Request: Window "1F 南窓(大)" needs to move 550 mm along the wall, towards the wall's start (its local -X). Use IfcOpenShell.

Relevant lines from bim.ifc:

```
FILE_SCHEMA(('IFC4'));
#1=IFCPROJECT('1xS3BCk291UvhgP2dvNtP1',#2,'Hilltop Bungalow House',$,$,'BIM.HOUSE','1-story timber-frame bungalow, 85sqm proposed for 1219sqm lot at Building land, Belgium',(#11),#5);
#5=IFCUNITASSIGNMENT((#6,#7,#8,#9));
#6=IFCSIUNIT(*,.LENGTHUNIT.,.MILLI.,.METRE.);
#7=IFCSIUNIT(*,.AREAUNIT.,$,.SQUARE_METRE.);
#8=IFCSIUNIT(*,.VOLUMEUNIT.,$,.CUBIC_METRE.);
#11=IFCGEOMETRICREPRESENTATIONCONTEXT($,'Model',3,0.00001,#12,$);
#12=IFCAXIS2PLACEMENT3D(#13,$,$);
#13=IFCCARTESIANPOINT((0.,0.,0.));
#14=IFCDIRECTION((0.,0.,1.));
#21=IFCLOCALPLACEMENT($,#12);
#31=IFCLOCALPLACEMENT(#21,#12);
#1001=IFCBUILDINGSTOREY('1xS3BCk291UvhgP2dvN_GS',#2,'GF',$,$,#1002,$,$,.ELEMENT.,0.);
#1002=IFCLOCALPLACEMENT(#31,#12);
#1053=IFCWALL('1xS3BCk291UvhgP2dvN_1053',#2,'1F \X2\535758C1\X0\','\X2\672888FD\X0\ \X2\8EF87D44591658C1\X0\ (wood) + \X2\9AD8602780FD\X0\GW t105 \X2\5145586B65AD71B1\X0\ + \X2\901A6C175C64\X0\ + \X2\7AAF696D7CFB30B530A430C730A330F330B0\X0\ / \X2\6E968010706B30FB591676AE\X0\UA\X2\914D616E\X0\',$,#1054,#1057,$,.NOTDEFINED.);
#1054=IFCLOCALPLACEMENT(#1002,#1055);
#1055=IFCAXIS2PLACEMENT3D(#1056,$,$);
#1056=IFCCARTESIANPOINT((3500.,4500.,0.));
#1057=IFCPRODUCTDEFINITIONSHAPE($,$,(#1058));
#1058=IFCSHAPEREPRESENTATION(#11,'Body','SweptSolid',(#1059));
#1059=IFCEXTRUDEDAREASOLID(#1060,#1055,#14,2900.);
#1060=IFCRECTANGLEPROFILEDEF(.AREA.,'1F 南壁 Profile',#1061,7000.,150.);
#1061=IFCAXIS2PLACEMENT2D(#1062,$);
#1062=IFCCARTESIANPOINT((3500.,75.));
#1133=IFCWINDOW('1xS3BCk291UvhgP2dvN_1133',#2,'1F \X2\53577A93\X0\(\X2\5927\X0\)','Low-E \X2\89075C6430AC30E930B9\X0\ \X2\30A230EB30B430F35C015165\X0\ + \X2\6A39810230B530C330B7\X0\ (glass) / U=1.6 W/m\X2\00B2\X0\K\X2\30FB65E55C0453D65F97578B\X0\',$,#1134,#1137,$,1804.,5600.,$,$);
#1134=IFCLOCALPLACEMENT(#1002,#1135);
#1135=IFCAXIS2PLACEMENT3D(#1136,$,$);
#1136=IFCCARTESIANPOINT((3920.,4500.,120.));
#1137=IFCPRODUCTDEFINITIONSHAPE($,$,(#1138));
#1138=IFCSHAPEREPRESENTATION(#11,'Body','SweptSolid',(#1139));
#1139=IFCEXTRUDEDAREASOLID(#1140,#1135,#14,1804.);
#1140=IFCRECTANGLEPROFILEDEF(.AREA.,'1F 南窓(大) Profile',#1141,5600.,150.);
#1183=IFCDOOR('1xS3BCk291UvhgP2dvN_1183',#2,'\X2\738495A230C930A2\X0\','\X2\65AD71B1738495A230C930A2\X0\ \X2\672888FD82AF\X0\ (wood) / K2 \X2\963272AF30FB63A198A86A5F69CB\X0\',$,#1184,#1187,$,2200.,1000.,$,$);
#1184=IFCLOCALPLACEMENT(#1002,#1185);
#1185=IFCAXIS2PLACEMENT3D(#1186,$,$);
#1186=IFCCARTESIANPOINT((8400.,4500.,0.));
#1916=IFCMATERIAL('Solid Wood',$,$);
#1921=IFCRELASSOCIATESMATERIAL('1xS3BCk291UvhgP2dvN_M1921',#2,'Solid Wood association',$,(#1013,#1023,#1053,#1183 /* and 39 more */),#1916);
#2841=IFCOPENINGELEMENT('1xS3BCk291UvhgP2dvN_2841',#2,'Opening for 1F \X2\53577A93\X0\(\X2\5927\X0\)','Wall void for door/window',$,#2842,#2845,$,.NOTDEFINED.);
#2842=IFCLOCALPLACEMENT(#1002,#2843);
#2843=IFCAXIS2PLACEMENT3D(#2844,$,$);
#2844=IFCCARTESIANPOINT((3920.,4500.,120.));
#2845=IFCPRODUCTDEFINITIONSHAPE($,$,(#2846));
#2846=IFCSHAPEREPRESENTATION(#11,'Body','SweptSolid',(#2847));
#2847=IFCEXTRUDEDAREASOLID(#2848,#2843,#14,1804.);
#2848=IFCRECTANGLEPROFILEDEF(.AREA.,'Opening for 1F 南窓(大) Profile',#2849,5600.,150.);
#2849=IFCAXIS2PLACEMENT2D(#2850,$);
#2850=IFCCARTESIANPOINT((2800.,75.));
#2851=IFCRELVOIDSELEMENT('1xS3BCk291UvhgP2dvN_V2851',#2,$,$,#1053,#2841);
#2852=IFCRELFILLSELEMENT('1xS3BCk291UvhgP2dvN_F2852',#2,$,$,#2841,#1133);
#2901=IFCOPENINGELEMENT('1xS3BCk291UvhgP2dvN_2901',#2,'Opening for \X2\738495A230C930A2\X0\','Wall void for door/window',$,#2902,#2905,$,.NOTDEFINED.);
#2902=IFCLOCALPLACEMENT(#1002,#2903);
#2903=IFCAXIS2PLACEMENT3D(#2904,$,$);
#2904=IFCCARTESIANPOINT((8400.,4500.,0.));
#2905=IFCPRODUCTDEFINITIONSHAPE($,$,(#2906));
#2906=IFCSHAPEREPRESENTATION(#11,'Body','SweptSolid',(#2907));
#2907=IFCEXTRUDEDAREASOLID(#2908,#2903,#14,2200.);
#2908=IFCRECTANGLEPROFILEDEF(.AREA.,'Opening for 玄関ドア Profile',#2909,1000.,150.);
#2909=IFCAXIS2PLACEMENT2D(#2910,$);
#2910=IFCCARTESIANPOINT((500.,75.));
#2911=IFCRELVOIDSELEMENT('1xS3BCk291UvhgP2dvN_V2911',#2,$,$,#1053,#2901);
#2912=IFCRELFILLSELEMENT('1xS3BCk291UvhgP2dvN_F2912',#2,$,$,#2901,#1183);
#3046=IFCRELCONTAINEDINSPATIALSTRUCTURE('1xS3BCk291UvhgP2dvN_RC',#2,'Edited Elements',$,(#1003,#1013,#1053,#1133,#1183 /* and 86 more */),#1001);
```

```python
import ifcopenshell
import ifcopenshell.api.geometry
import ifcopenshell.util.placement

model = ifcopenshell.open("bim.ifc")

window = model.by_guid("1xS3BCk291UvhgP2dvN_1133")
opening = window.FillsVoids[0].RelatingOpeningElement
wall = opening.VoidsElements[0].RelatingBuildingElement

wall_matrix = ifcopenshell.util.placement.get_local_placement(wall.ObjectPlacement)
shift = wall_matrix[:3, 0] * -550.0
before = ifcopenshell.util.placement.get_local_placement(window.ObjectPlacement)[:3, 3].copy()

# The window is not placed relative to its opening, so move both.
for product in (opening, window):
    matrix = ifcopenshell.util.placement.get_local_placement(product.ObjectPlacement)
    matrix[:3, 3] += shift
    ifcopenshell.api.geometry.edit_object_placement(model, product=product, matrix=matrix, is_si=False)

after = ifcopenshell.util.placement.get_local_placement(window.ObjectPlacement)[:3, 3]
print("window moved by", (after - before).round(3) + 0.0)

model.write("bim-out.ifc")
```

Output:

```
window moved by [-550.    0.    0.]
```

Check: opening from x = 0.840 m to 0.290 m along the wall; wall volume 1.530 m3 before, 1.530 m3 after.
